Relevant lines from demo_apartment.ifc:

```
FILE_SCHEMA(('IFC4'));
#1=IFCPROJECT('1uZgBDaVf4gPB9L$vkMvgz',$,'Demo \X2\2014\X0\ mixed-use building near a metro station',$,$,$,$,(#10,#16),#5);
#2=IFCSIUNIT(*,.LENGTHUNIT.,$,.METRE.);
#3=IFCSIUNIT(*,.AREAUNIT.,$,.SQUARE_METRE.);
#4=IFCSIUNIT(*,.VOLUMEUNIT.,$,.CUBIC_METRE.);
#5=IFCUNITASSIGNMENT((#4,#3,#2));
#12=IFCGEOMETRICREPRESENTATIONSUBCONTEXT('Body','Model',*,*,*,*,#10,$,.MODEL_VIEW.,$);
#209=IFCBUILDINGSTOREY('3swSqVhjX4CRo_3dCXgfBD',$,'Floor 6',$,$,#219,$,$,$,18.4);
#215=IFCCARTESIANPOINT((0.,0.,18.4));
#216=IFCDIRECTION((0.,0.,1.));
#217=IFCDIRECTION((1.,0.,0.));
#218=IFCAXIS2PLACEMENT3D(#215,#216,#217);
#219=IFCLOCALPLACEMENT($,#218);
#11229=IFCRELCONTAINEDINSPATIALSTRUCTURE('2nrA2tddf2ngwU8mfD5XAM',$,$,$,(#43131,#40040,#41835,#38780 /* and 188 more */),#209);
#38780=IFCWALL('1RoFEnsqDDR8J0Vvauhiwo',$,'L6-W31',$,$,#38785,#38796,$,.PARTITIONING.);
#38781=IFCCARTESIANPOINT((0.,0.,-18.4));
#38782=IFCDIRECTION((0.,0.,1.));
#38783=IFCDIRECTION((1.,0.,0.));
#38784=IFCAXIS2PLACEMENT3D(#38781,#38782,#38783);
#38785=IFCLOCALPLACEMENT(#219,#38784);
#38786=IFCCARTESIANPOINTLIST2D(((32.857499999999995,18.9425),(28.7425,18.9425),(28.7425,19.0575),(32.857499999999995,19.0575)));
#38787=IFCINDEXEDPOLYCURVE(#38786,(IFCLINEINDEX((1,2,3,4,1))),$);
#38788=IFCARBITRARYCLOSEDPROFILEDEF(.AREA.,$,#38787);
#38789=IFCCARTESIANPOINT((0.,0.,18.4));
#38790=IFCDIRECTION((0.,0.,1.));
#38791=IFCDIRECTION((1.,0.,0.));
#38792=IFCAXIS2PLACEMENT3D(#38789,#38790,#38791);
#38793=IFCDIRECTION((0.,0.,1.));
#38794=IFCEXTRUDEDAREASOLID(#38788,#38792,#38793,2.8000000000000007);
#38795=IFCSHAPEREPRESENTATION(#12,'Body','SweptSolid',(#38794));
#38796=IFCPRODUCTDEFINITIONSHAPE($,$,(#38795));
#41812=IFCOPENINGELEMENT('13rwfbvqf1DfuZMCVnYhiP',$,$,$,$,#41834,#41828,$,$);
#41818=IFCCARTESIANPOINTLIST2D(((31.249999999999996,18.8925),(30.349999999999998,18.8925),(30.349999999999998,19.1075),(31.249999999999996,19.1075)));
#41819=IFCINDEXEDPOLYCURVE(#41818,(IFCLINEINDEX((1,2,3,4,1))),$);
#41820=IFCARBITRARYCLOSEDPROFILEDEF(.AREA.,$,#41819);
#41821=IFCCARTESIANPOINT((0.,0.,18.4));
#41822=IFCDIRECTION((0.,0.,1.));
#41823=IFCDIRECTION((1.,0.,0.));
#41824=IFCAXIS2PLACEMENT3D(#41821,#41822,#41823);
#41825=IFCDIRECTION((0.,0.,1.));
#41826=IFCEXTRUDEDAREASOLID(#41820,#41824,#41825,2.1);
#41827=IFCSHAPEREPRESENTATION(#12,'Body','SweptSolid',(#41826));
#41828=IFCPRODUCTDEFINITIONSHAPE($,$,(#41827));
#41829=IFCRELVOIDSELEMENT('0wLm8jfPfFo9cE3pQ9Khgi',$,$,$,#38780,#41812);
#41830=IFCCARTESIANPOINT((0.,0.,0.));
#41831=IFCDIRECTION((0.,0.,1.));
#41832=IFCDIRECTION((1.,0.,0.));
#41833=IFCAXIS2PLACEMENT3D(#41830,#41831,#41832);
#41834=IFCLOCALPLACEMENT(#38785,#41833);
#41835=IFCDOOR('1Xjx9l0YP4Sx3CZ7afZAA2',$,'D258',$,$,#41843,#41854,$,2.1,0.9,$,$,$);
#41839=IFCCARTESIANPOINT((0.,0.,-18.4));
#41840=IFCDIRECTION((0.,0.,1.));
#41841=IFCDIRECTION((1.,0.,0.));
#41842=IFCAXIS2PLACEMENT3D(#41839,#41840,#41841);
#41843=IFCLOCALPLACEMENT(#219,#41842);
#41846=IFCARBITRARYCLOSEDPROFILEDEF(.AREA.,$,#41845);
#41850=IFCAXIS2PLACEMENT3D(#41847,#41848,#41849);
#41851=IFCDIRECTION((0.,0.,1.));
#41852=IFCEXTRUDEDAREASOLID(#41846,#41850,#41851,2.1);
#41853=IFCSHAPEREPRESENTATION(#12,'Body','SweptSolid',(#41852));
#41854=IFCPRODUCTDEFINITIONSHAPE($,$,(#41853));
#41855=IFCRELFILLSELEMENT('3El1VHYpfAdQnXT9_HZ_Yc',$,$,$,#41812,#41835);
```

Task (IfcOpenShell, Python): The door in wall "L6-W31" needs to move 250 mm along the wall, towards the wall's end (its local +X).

```python
import ifcopenshell
import ifcopenshell.api.geometry
import ifcopenshell.util.placement
import ifcopenshell.util.unit

model = ifcopenshell.open("demo_apartment.ifc")
unit_scale = ifcopenshell.util.unit.calculate_unit_scale(model)

door = model.by_guid("1Xjx9l0YP4Sx3CZ7afZAA2")
opening = door.FillsVoids[0].RelatingOpeningElement
wall = opening.VoidsElements[0].RelatingBuildingElement

wall_matrix = ifcopenshell.util.placement.get_local_placement(wall.ObjectPlacement)
shift = wall_matrix[:3, 0] * 0.25 / unit_scale
before = ifcopenshell.util.placement.get_local_placement(door.ObjectPlacement)[:3, 3].copy()

# The door is not placed relative to its opening, so move both.
for product in (opening, door):
    matrix = ifcopenshell.util.placement.get_local_placement(product.ObjectPlacement)
    matrix[:3, 3] += shift
    ifcopenshell.api.geometry.edit_object_placement(model, product=product, matrix=matrix, is_si=False)

after = ifcopenshell.util.placement.get_local_placement(door.ObjectPlacement)[:3, 3]
print("door moved by", (after - before).round(3) + 0.0)

model.write("demo_apartment-out.ifc")
```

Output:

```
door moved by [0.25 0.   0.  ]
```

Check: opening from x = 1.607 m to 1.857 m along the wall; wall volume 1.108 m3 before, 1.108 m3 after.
